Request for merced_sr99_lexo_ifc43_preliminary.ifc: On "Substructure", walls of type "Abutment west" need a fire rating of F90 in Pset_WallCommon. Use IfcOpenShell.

First a look at what the model holds.

```python
import ifcopenshell
import ifcopenshell.util.element

model = ifcopenshell.open("merced_sr99_lexo_ifc43_preliminary.ifc")
print(model.schema)
storey = next(s for s in model.by_type("IfcBuildingStorey") if s.Name == "Substructure")
walls = [e for e in ifcopenshell.util.element.get_decomposition(storey) if e.is_a("IfcWall")]
seen = {}
for e in walls:
    element_type = ifcopenshell.util.element.get_type(e)
    key = (element_type.Name if element_type != e and element_type else None, ifcopenshell.util.element.get_pset(e, "Pset_WallCommon", "FireRating"))
    seen[key] = seen.get(key, 0) + 1
for (name, value), count in sorted(seen.items(), key=str):
    print(count, "x", name, "|", value)
```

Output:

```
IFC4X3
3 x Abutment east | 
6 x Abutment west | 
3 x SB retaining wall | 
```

```python
import ifcopenshell
import ifcopenshell.api.pset
import ifcopenshell.util.element

model = ifcopenshell.open("merced_sr99_lexo_ifc43_preliminary.ifc")

storey = next(s for s in model.by_type("IfcBuildingStorey") if s.Name == "Substructure")
walls = [e for e in ifcopenshell.util.element.get_decomposition(storey) if e.is_a("IfcWall")]

count = 0
for e in walls:
    element_type = ifcopenshell.util.element.get_type(e)
    if element_type in (None, e) or element_type.Name != "Abutment west":
        continue
    # add_pset returns the element's existing set when there is one.
    pset = ifcopenshell.api.pset.add_pset(model, product=e, name="Pset_WallCommon")
    ifcopenshell.api.pset.edit_pset(model, pset=pset, properties={"FireRating": "F90"})
    count += 1

print(count, "walls updated")

model.write("merced_sr99_lexo_ifc43_preliminary_updated.ifc")
```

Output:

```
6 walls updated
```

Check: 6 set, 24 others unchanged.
